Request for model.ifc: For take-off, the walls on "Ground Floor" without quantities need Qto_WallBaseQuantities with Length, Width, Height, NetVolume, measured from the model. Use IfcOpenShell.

First a look at what the model holds.

```python
import ifcopenshell
import ifcopenshell.util.element
import ifcopenshell.util.unit

model = ifcopenshell.open("model.ifc")
print(model.schema)
for unit_type in ("LENGTHUNIT", "AREAUNIT", "VOLUMEUNIT"):
    print(unit_type, ifcopenshell.util.unit.calculate_unit_scale(model, unit_type))
storey = next(s for s in model.by_type("IfcBuildingStorey") if s.Name == "Ground Floor")
walls = [e for e in ifcopenshell.util.element.get_decomposition(storey) if e.is_a("IfcWall")]
for e in sorted(walls, key=lambda e: e.id()):
    print(e.id(), e.is_a(), e.Name, list(ifcopenshell.util.element.get_psets(e, qtos_only=True)), sep=" | ")
```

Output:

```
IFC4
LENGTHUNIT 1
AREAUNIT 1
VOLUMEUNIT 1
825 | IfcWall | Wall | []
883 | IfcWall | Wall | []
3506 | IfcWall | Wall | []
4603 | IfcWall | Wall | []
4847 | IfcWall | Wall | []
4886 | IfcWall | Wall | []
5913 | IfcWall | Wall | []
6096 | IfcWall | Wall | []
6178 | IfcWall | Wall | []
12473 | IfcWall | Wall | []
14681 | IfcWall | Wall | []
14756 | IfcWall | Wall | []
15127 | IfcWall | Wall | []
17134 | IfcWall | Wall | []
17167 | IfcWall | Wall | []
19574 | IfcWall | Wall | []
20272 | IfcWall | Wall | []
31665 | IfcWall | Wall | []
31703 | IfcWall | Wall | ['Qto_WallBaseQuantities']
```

```python
import ifcopenshell
import ifcopenshell.api.pset
import ifcopenshell.geom
import ifcopenshell.util.element
import ifcopenshell.util.shape
import ifcopenshell.util.unit

model = ifcopenshell.open("model.ifc")
unit_scale = ifcopenshell.util.unit.calculate_unit_scale(model)
volume_scale = ifcopenshell.util.unit.calculate_unit_scale(model, "VOLUMEUNIT")
settings = ifcopenshell.geom.settings()

storey = next(s for s in model.by_type("IfcBuildingStorey") if s.Name == "Ground Floor")
walls = [e for e in ifcopenshell.util.element.get_decomposition(storey) if e.is_a("IfcWall")]

for e in sorted(walls, key=lambda e: e.id()):
    if ifcopenshell.util.element.get_psets(e, qtos_only=True, should_inherit=False):
        continue
    # Geometry comes back in metres, in the element's own axes.
    shape = ifcopenshell.geom.create_shape(settings, e)
    values = {
        "Length": ifcopenshell.util.shape.get_x(shape.geometry) / unit_scale,
        "Width": ifcopenshell.util.shape.get_y(shape.geometry) / unit_scale,
        "Height": ifcopenshell.util.shape.get_z(shape.geometry) / unit_scale,
        "NetVolume": ifcopenshell.util.shape.get_volume(shape.geometry) / volume_scale,
    }
    qto = ifcopenshell.api.pset.add_qto(model, product=e, name="Qto_WallBaseQuantities")
    ifcopenshell.api.pset.edit_qto(model, qto=qto, properties=values)
    print(e.id(), {k: round(v, 3) for k, v in values.items()})

model.write("model_v2.ifc")
```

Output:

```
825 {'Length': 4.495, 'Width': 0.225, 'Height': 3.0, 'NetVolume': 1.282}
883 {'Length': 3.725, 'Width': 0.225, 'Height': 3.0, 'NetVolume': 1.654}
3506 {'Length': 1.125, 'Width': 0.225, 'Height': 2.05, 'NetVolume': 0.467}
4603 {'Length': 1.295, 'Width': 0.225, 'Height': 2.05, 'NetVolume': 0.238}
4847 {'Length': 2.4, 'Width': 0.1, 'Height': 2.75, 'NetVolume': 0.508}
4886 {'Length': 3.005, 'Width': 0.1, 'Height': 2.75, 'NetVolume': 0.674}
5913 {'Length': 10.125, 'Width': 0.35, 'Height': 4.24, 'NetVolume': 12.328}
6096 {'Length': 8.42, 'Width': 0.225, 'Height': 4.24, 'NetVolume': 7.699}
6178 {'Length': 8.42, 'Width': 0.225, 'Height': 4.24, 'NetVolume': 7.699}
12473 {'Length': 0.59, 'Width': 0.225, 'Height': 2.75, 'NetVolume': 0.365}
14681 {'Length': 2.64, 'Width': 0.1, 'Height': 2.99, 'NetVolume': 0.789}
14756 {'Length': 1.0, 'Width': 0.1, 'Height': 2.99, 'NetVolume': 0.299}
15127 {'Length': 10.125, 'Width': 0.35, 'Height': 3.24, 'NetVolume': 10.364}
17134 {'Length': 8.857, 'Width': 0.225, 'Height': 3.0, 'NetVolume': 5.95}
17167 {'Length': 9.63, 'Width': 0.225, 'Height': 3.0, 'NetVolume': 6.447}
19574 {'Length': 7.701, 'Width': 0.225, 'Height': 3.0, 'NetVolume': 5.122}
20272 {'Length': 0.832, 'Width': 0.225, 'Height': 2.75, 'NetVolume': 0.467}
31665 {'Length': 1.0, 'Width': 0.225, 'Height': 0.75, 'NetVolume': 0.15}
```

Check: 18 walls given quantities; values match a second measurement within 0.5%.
